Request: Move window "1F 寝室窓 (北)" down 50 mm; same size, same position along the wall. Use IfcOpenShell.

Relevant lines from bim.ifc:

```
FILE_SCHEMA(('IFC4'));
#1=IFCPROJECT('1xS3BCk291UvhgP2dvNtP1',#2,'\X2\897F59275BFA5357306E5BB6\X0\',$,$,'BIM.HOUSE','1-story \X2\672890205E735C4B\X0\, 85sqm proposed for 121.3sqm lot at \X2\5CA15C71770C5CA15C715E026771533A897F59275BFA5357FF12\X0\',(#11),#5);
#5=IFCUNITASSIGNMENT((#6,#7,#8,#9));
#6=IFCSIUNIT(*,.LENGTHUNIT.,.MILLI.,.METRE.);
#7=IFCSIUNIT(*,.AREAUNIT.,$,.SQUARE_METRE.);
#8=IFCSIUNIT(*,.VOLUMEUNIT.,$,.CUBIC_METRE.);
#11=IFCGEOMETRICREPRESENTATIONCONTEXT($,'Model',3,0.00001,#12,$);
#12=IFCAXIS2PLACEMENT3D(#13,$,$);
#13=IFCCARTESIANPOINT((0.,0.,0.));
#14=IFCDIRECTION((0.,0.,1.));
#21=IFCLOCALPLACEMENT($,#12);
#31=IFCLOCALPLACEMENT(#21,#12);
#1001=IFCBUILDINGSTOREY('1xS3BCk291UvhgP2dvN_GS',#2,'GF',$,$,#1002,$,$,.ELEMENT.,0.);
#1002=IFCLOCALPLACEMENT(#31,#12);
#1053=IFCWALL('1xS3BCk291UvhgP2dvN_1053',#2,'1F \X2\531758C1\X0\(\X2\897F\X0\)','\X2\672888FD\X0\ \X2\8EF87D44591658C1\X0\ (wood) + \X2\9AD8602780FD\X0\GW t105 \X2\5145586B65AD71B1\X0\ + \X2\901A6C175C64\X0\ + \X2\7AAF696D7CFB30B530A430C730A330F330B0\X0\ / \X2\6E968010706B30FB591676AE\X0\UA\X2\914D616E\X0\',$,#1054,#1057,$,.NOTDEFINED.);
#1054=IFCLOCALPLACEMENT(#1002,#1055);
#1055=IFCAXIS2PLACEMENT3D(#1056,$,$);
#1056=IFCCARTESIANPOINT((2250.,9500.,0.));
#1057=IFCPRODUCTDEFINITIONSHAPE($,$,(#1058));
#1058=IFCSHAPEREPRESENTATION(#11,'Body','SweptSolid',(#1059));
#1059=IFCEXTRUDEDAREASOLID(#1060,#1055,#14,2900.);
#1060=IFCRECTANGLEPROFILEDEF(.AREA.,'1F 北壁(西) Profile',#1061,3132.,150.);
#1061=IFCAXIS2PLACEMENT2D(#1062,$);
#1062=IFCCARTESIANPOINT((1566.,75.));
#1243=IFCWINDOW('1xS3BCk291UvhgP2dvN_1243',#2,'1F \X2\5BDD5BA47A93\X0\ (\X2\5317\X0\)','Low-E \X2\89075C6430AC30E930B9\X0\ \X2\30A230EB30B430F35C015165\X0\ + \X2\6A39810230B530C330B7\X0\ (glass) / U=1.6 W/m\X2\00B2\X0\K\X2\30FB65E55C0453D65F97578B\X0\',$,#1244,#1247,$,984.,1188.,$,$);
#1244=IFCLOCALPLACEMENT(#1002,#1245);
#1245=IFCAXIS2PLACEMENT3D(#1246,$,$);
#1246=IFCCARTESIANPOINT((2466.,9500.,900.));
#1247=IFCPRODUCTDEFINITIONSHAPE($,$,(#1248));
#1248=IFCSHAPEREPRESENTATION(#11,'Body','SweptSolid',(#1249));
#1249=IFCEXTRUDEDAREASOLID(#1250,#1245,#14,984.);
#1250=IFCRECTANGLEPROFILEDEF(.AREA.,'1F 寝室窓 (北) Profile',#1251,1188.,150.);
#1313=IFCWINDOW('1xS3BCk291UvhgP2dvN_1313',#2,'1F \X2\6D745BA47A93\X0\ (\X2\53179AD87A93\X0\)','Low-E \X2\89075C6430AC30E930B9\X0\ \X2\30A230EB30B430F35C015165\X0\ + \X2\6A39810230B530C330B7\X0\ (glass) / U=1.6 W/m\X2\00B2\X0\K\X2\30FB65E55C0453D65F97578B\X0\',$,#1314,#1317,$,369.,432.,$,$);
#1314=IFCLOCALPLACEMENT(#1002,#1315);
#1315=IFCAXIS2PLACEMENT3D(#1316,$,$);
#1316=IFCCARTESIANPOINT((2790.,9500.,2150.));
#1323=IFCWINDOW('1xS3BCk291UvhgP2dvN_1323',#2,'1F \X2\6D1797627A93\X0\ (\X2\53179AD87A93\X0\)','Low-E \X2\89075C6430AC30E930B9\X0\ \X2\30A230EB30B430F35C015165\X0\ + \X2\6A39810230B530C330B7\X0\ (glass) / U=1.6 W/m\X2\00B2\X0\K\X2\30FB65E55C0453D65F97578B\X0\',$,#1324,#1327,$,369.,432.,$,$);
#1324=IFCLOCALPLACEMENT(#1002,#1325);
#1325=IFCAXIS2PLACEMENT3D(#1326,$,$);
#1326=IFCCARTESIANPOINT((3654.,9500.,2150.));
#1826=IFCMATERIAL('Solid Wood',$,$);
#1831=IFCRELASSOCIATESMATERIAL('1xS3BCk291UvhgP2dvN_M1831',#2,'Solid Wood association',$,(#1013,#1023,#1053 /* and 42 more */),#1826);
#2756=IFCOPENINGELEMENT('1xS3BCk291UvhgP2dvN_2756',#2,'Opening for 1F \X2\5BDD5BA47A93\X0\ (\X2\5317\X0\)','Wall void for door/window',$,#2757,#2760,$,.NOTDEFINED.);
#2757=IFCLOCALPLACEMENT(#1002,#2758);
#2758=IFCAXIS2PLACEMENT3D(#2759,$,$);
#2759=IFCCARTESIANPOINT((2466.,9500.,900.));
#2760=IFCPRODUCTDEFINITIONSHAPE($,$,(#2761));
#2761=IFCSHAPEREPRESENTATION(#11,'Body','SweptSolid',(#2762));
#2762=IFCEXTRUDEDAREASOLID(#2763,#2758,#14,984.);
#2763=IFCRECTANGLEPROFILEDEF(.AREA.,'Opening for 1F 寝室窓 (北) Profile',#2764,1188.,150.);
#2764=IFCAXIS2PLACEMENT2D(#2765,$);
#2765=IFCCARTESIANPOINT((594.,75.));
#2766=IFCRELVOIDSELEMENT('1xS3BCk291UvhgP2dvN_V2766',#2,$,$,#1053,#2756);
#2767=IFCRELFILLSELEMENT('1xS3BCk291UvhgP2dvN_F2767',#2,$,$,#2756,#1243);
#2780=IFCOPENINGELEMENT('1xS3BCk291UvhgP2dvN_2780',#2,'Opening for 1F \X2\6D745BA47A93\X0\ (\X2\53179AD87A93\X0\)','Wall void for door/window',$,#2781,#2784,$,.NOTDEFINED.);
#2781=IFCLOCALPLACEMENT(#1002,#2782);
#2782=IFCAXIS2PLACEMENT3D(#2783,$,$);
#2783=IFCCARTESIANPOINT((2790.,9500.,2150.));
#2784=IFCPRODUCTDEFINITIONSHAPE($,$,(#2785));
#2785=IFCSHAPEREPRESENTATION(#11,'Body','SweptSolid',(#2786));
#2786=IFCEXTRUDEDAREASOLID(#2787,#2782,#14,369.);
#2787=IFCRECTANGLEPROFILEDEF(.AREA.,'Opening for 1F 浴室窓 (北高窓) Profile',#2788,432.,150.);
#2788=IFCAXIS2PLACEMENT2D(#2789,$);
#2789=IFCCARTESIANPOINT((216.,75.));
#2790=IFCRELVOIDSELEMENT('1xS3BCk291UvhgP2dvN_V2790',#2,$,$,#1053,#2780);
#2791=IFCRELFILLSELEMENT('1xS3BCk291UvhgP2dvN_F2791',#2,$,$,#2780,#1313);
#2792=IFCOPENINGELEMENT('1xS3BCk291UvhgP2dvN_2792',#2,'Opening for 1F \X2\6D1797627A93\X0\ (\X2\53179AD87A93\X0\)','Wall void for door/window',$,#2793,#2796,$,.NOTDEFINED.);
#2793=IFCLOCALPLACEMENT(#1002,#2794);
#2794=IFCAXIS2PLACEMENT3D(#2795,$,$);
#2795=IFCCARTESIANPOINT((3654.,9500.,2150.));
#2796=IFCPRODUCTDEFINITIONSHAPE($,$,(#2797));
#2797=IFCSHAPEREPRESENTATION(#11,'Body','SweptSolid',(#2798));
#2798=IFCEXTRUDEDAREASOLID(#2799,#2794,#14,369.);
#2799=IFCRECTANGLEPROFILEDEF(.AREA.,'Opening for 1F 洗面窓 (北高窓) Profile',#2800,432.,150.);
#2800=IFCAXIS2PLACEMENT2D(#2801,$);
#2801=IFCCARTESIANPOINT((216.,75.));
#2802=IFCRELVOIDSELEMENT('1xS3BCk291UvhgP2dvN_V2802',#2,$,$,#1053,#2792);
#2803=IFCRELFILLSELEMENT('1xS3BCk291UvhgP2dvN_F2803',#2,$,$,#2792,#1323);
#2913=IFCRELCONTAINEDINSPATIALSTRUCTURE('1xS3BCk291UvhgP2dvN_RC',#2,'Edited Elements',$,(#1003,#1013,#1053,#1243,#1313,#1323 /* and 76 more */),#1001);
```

```python
import numpy as np
import ifcopenshell
import ifcopenshell.api.geometry
import ifcopenshell.util.placement
import ifcopenshell.util.unit

model = ifcopenshell.open("bim.ifc")
unit_scale = ifcopenshell.util.unit.calculate_unit_scale(model)

window = model.by_guid("1xS3BCk291UvhgP2dvN_1243")
opening = window.FillsVoids[0].RelatingOpeningElement
dz = -50.0

shift = np.array([0.0, 0.0, dz])
# The window is not placed relative to its opening, so move both.
for product in (opening, window):
    matrix = ifcopenshell.util.placement.get_local_placement(product.ObjectPlacement)
    matrix[:3, 3] += shift
    ifcopenshell.api.geometry.edit_object_placement(model, product=product, matrix=matrix, is_si=False)

print(f"moved by {dz * unit_scale:+.3f} m")

model.write("bim_edited.ifc")
```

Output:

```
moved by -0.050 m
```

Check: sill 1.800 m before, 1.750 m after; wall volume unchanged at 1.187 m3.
